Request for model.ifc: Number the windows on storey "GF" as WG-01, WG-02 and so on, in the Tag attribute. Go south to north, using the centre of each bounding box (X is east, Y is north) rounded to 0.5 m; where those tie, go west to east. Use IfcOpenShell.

First a look at what the model holds.

```python
import ifcopenshell
import ifcopenshell.util.element
import ifcopenshell.util.placement

model = ifcopenshell.open("model.ifc")
print(model.schema)
storey = next(s for s in model.by_type("IfcBuildingStorey") if s.Name == "GF")
windows = [e for e in ifcopenshell.util.element.get_decomposition(storey) if e.is_a("IfcWindow")]
for e in sorted(windows, key=lambda e: e.id()):
    origin = ifcopenshell.util.placement.get_local_placement(e.ObjectPlacement)[:3, 3]
    print(e.id(), e.Tag, e.Name, origin.round(2) + 0.0, sep=" | ")
```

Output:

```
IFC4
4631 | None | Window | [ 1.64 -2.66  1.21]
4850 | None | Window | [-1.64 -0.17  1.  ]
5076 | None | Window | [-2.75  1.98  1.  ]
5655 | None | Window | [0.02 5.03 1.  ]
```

```python
import ifcopenshell
import ifcopenshell.geom
import ifcopenshell.util.element
import ifcopenshell.util.shape

model = ifcopenshell.open("model.ifc")
settings = ifcopenshell.geom.settings()
settings.set("use-world-coords", True)


def centre(element):
    shape = ifcopenshell.geom.create_shape(settings, element)
    return ifcopenshell.util.shape.get_bbox_centroid(shape.geometry)


storey = next(s for s in model.by_type("IfcBuildingStorey") if s.Name == "GF")
windows = [e for e in ifcopenshell.util.element.get_decomposition(storey) if e.is_a("IfcWindow")]

# Insertion points can sit at a corner or the storey origin, so sort by the geometry (in metres).
centres = {e: centre(e) for e in windows}
windows.sort(key=lambda e: (round(centres[e][1] / 0.5), centres[e][0]))

for i, e in enumerate(windows, start=1):
    number = f"WG-{i:02d}"
    e.Tag = number
    print(e.id(), number)

model.write("model_updated.ifc")
```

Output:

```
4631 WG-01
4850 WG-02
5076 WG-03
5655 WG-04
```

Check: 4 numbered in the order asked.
